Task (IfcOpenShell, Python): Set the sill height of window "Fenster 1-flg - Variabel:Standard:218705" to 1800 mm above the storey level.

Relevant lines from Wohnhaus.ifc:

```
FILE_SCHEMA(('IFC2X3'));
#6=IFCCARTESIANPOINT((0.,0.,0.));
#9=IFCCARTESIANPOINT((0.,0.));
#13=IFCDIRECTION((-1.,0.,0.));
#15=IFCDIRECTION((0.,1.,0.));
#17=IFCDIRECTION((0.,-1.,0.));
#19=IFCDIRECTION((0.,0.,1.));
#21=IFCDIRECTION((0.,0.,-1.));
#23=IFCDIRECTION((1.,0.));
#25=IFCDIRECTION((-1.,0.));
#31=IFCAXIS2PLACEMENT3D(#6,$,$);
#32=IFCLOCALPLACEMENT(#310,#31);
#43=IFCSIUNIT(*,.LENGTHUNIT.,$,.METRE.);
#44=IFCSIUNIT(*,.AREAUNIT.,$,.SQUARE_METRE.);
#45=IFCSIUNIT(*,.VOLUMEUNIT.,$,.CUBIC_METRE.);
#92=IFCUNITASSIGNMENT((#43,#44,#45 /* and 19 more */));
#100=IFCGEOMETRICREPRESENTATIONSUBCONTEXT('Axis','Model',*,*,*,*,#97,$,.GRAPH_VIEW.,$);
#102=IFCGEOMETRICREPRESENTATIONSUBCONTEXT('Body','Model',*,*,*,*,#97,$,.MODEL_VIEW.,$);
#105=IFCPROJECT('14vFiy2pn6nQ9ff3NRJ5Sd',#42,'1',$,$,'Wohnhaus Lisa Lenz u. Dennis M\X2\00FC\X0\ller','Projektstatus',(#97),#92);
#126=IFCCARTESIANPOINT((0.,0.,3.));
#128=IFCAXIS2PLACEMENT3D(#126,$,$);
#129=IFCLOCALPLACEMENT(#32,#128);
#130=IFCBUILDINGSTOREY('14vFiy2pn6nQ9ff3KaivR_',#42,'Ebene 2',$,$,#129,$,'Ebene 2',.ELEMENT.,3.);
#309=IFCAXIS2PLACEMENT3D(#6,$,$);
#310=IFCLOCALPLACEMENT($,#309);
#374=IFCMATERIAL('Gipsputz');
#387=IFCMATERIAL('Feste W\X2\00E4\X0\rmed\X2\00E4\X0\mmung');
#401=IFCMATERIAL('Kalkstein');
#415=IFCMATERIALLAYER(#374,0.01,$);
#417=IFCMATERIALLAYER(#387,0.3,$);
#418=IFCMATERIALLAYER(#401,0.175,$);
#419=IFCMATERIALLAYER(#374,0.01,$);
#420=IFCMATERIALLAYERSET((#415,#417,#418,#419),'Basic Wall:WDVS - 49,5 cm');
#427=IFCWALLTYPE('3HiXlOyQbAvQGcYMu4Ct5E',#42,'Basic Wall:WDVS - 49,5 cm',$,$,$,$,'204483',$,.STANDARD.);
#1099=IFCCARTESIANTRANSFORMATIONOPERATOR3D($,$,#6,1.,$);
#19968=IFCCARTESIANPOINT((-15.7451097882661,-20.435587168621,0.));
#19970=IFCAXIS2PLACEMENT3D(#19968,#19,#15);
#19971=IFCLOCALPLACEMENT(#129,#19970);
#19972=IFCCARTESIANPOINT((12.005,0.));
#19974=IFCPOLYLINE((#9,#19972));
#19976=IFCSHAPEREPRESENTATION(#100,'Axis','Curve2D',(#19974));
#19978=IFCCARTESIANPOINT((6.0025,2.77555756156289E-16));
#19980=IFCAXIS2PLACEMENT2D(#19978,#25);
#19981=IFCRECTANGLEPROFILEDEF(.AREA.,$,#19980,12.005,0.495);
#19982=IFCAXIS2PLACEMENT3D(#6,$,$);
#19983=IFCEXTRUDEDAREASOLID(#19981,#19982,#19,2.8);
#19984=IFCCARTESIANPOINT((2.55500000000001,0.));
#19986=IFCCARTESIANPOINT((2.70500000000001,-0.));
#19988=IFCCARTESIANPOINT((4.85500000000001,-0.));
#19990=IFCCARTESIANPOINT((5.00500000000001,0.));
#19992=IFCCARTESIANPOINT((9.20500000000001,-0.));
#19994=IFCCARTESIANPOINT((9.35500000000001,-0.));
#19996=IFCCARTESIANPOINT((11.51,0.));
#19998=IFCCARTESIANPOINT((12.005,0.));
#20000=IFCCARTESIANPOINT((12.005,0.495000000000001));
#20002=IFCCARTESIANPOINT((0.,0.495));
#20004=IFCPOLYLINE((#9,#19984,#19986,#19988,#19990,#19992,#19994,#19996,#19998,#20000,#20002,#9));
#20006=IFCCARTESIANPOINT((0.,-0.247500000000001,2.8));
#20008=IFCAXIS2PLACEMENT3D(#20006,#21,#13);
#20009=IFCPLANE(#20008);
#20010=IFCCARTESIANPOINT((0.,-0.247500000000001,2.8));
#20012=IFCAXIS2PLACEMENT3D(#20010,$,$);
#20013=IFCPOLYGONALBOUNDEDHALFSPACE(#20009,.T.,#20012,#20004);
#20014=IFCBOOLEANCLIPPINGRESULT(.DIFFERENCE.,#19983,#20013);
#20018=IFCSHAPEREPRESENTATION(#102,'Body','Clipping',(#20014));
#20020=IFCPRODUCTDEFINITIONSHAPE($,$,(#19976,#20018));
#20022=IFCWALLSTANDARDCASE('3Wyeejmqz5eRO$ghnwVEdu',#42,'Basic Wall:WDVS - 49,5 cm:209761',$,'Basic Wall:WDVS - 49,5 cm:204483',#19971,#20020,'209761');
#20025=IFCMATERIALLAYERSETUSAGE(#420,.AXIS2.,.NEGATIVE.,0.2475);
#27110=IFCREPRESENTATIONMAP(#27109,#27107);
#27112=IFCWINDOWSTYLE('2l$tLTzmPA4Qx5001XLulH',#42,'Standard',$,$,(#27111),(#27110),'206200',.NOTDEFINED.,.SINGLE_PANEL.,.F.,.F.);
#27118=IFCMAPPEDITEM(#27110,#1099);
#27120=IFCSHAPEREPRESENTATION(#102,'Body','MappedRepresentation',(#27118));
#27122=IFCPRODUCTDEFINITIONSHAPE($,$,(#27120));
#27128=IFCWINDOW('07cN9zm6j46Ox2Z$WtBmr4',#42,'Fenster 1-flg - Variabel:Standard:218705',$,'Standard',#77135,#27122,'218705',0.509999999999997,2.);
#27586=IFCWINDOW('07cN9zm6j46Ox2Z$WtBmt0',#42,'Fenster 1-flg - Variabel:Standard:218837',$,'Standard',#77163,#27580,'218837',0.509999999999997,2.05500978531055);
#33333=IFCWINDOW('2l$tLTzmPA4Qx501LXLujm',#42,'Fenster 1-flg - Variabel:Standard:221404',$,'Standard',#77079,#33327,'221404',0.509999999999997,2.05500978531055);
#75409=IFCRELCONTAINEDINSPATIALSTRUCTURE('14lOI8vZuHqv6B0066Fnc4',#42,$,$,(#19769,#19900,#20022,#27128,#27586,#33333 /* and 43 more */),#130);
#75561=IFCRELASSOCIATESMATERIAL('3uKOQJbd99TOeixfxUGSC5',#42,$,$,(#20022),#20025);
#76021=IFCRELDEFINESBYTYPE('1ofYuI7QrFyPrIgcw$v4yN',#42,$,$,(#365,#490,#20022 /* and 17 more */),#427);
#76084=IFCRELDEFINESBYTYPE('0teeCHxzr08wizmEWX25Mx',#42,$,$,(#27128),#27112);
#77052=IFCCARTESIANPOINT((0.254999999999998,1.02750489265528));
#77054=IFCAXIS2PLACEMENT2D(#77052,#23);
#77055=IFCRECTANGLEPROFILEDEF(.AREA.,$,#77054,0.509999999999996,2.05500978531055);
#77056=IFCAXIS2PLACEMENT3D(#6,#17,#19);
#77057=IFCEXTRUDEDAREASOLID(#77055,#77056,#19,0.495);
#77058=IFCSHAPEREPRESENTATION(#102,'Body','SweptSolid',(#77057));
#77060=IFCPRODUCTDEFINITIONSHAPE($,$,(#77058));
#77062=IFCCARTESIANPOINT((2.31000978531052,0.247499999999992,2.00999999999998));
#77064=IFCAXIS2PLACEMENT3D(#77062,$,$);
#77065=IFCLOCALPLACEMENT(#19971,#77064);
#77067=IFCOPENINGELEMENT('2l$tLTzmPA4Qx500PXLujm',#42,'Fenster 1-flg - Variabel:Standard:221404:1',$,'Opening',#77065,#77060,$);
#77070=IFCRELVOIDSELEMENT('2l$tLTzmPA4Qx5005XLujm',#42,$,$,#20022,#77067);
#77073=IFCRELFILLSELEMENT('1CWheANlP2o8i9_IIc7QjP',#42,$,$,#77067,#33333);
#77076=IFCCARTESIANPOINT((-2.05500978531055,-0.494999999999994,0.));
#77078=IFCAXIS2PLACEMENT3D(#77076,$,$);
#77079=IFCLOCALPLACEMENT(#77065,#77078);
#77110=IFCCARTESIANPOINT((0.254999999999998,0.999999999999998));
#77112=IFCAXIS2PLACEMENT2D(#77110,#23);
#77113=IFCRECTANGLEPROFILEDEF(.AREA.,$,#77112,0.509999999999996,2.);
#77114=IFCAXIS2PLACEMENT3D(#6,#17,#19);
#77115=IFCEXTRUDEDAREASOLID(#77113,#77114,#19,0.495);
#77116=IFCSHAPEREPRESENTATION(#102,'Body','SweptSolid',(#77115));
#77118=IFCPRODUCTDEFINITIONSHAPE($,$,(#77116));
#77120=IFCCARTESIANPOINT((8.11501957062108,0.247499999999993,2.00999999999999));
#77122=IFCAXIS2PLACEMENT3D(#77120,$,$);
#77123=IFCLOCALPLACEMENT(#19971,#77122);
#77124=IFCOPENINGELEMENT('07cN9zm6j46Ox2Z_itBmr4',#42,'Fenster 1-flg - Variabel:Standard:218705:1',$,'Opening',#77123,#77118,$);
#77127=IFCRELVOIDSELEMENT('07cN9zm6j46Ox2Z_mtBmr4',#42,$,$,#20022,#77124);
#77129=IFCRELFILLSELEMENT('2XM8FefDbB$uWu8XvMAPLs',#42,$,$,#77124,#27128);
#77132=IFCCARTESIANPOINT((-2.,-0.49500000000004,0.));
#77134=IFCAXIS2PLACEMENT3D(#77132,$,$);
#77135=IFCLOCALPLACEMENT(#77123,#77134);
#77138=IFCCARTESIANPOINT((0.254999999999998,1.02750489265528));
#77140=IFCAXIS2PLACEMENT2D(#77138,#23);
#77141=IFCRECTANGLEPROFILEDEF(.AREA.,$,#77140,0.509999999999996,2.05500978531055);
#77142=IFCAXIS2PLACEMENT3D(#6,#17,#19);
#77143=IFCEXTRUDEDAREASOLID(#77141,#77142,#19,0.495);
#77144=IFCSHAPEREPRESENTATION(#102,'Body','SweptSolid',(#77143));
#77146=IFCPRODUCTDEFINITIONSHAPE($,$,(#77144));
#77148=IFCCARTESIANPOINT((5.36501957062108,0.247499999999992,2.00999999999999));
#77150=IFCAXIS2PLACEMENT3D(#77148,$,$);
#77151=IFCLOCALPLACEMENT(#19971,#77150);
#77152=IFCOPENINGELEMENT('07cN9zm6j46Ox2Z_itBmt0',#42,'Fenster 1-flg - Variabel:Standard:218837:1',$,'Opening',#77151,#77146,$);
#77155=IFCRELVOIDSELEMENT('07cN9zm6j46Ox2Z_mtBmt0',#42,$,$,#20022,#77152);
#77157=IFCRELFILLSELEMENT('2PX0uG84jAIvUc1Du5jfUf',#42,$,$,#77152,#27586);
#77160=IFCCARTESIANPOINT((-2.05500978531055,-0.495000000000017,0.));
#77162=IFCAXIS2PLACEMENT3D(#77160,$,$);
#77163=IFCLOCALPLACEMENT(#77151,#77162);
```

```python
import numpy as np
import ifcopenshell
import ifcopenshell.api.geometry
import ifcopenshell.geom
import ifcopenshell.util.element
import ifcopenshell.util.placement
import ifcopenshell.util.shape
import ifcopenshell.util.unit

model = ifcopenshell.open("Wohnhaus.ifc")
unit_scale = ifcopenshell.util.unit.calculate_unit_scale(model)

window = model.by_id(27128)
opening = window.FillsVoids[0].RelatingOpeningElement
storey = ifcopenshell.util.element.get_container(window, ifc_class="IfcBuildingStorey")
level = ifcopenshell.util.placement.get_local_placement(storey.ObjectPlacement)[2, 3]

# The opening's origin need not be at the sill, so measure its lowest point.
shape = ifcopenshell.geom.create_shape(ifcopenshell.geom.settings(), opening)
bottom = ifcopenshell.util.shape.get_shape_bottom_elevation(shape, shape.geometry) / unit_scale
dz = level + 1.8 / unit_scale - bottom

shift = np.array([0.0, 0.0, dz])
# The window is placed relative to its opening, so it follows when the opening moves.
matrix = ifcopenshell.util.placement.get_local_placement(opening.ObjectPlacement)
matrix[:3, 3] += shift
ifcopenshell.api.geometry.edit_object_placement(
    model, product=opening, matrix=matrix, is_si=False, should_transform_children=True
)

print(f"moved by {dz * unit_scale:+.3f} m")

model.write("Wohnhaus_edited.ifc")
```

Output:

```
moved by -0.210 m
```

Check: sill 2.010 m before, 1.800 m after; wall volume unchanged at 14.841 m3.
